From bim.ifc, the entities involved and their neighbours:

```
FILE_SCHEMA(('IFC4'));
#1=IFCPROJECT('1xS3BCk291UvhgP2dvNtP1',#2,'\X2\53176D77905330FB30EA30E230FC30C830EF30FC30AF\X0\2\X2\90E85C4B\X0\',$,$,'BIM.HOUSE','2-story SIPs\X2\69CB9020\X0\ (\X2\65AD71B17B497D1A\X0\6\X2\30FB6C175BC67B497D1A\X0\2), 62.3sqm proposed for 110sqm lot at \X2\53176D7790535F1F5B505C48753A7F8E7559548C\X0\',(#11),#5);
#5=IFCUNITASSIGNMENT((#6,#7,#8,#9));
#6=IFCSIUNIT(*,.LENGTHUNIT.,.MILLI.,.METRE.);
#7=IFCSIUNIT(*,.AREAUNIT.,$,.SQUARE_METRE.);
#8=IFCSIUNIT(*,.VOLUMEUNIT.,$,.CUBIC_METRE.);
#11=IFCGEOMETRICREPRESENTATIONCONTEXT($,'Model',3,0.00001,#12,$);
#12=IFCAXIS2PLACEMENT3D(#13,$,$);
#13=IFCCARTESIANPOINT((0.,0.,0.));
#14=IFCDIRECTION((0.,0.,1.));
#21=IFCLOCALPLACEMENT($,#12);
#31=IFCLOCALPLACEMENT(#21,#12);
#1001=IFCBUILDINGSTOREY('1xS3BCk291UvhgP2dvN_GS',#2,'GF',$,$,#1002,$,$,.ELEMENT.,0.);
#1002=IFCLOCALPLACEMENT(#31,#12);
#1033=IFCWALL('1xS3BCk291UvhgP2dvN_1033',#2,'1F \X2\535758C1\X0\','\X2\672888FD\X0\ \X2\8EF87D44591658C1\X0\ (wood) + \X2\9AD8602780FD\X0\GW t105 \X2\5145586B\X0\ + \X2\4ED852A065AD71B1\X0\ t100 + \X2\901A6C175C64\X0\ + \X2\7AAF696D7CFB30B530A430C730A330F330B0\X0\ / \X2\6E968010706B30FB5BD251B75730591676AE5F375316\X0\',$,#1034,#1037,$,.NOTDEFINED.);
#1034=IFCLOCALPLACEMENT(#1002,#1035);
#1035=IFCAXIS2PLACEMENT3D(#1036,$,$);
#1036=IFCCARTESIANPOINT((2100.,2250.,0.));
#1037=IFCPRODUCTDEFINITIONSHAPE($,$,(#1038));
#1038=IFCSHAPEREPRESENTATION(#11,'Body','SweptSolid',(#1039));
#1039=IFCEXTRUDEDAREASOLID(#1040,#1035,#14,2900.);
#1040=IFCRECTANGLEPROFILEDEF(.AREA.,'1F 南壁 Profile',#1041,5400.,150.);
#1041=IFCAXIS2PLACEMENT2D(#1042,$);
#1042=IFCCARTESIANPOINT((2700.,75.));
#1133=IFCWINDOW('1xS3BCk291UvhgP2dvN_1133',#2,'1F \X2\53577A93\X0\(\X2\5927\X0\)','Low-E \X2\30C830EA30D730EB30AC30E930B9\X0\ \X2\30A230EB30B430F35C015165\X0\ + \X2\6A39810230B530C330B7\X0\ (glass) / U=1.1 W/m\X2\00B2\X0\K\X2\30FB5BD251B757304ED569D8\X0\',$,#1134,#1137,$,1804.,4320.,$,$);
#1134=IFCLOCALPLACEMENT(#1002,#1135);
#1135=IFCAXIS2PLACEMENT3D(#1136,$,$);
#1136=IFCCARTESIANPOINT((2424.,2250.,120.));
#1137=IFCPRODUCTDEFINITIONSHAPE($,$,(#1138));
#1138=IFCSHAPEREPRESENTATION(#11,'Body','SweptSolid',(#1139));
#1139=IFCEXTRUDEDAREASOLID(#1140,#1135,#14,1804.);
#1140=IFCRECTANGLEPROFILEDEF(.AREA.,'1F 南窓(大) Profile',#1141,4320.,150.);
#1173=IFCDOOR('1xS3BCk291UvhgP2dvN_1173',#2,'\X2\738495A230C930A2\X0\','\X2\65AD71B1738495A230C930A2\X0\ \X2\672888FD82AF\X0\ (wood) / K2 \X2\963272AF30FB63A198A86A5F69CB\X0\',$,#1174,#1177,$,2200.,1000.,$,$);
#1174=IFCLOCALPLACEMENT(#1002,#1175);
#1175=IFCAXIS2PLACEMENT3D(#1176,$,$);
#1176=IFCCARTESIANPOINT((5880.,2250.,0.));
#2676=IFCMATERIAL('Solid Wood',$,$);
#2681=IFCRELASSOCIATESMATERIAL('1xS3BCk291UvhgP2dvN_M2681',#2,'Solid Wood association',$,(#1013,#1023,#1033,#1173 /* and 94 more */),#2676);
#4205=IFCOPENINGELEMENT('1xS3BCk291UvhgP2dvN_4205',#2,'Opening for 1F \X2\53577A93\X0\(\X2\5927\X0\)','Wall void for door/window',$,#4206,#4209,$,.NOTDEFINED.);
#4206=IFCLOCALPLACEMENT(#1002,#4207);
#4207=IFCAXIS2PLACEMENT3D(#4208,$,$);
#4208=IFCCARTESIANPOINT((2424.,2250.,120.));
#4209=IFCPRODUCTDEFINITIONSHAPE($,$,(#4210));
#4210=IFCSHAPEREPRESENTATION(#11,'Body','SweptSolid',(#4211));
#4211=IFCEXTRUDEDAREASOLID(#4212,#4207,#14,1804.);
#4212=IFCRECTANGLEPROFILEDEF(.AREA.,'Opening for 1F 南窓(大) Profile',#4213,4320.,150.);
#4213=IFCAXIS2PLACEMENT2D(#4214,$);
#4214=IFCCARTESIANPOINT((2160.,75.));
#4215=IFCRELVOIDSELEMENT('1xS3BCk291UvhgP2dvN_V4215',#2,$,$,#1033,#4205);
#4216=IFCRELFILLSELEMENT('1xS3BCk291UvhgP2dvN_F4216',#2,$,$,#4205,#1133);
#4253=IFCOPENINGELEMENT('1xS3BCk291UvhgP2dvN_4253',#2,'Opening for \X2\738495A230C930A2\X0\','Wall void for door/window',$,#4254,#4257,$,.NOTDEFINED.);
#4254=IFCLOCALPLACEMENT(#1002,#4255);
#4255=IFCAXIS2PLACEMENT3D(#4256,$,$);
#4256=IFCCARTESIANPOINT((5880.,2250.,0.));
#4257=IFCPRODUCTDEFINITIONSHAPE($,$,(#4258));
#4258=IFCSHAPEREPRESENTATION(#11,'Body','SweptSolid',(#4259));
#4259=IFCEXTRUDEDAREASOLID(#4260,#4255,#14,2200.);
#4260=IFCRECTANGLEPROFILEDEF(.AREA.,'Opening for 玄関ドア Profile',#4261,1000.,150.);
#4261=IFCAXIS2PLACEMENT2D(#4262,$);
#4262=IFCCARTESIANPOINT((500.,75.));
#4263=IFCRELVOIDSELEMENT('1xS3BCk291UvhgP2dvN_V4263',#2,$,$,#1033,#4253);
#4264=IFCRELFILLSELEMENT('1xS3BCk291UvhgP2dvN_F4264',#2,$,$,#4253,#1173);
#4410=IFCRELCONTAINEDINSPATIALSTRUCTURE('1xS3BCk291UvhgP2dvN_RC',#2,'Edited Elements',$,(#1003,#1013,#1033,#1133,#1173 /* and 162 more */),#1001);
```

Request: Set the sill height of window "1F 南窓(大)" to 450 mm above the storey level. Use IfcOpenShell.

```python
import numpy as np
import ifcopenshell
import ifcopenshell.api.geometry
import ifcopenshell.geom
import ifcopenshell.util.element
import ifcopenshell.util.placement
import ifcopenshell.util.shape
import ifcopenshell.util.unit

model = ifcopenshell.open("bim.ifc")
unit_scale = ifcopenshell.util.unit.calculate_unit_scale(model)

window = model.by_id(1133)
opening = window.FillsVoids[0].RelatingOpeningElement
storey = ifcopenshell.util.element.get_container(window, ifc_class="IfcBuildingStorey")
level = ifcopenshell.util.placement.get_local_placement(storey.ObjectPlacement)[2, 3]

# The opening's origin need not be at the sill, so measure its lowest point.
shape = ifcopenshell.geom.create_shape(ifcopenshell.geom.settings(), opening)
bottom = ifcopenshell.util.shape.get_shape_bottom_elevation(shape, shape.geometry) / unit_scale
dz = level + 0.45 / unit_scale - bottom

shift = np.array([0.0, 0.0, dz])
# The window is not placed relative to its opening, so move both.
for product in (opening, window):
    matrix = ifcopenshell.util.placement.get_local_placement(product.ObjectPlacement)
    matrix[:3, 3] += shift
    ifcopenshell.api.geometry.edit_object_placement(model, product=product, matrix=matrix, is_si=False)

print(f"moved by {dz * unit_scale:+.3f} m")

model.write("bim_edited.ifc")
```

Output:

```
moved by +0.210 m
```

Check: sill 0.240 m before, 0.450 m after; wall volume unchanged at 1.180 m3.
